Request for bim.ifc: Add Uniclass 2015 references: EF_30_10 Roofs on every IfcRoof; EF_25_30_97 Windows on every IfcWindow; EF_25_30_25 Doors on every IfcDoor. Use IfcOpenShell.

First a look at what the model holds.

```python
import ifcopenshell

model = ifcopenshell.open("bim.ifc")
print(model.schema)
print("classifications:", [c.Name for c in model.by_type("IfcClassification")])
for ifc_class in ("IfcDoor", "IfcRoof", "IfcStair", "IfcWall", "IfcWindow"):
    print(ifc_class, len(model.by_type(ifc_class)))
```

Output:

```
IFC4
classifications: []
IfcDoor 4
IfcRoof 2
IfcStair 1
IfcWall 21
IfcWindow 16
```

```python
import ifcopenshell
import ifcopenshell.api.classification

model = ifcopenshell.open("bim.ifc")

system = ifcopenshell.api.classification.add_classification(model, classification="Uniclass 2015")

codes = {
    "IfcRoof": ("EF_30_10", "Roofs"),
    "IfcWindow": ("EF_25_30_97", "Windows"),
    "IfcDoor": ("EF_25_30_25", "Doors"),
}
for ifc_class, (code, name) in codes.items():
    products = model.by_type(ifc_class)
    ifcopenshell.api.classification.add_reference(
        model, products=products, classification=system, identification=code, name=name
    )
    print(code, len(products))

model.write("bim_edited.ifc")
```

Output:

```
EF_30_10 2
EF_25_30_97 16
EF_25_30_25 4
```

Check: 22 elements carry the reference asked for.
